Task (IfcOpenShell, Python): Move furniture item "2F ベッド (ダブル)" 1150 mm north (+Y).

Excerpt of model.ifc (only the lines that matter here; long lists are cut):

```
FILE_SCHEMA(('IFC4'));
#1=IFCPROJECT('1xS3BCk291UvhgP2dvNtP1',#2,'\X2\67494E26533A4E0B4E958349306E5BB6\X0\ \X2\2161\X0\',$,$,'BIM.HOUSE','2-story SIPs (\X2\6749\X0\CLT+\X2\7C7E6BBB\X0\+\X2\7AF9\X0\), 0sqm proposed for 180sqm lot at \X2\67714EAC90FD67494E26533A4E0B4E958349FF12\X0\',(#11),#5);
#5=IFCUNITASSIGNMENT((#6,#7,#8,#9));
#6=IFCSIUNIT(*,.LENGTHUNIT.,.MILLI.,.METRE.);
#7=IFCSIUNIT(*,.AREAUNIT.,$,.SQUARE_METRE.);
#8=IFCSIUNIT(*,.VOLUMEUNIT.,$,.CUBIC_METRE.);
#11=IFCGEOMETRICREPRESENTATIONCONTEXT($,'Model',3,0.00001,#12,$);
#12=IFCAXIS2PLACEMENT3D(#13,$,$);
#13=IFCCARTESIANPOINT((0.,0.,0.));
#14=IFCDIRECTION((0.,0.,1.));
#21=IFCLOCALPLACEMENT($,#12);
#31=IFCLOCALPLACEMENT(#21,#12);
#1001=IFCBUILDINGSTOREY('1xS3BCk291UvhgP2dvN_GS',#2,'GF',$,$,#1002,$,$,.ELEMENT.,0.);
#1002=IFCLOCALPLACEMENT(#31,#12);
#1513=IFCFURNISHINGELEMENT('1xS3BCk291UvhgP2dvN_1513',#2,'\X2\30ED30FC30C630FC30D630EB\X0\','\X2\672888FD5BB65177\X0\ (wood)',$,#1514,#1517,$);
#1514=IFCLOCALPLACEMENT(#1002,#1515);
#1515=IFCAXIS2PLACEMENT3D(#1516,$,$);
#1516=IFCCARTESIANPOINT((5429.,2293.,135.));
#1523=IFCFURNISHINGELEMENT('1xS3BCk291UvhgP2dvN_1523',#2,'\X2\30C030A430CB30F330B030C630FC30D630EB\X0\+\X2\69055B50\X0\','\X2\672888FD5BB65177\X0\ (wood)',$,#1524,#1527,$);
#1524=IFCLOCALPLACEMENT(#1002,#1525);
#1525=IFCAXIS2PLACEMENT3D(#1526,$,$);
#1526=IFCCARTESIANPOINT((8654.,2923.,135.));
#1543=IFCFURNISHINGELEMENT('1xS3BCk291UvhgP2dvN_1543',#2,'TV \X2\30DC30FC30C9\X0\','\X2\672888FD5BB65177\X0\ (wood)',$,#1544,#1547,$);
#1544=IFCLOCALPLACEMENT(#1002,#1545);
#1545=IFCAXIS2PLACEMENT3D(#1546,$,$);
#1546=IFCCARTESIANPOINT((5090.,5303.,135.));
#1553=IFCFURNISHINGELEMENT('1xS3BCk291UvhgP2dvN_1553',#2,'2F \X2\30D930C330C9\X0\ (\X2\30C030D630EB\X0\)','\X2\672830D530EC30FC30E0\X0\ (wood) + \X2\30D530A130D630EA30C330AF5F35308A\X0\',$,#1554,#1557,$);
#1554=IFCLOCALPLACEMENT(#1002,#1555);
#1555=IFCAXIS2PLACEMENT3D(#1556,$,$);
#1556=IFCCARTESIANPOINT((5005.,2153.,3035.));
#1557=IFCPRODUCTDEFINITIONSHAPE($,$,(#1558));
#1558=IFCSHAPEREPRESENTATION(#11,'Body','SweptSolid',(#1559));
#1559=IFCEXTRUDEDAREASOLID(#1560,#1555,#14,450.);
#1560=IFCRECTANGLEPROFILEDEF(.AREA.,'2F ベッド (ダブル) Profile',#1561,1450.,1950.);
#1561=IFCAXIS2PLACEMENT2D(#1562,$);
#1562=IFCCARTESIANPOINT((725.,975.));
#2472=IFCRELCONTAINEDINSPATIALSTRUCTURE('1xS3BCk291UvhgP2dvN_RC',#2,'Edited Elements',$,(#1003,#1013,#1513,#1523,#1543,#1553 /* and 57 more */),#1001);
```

```python
import ifcopenshell
import ifcopenshell.api.geometry
import ifcopenshell.util.placement
import ifcopenshell.util.unit

model = ifcopenshell.open("model.ifc")
unit_scale = ifcopenshell.util.unit.calculate_unit_scale(model)

item = model.by_id(1553)
matrix = ifcopenshell.util.placement.get_local_placement(item.ObjectPlacement)
matrix[1, 3] += 1.15 / unit_scale
ifcopenshell.api.geometry.edit_object_placement(model, product=item, matrix=matrix, is_si=False)

print(ifcopenshell.util.placement.get_local_placement(item.ObjectPlacement).round(3) + 0.0)

model.write("model_updated.ifc")
```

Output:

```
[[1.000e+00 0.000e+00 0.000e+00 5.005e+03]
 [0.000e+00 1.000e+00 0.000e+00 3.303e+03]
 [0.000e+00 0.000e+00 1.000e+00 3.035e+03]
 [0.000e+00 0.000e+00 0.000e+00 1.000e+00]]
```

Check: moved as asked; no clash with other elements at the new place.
